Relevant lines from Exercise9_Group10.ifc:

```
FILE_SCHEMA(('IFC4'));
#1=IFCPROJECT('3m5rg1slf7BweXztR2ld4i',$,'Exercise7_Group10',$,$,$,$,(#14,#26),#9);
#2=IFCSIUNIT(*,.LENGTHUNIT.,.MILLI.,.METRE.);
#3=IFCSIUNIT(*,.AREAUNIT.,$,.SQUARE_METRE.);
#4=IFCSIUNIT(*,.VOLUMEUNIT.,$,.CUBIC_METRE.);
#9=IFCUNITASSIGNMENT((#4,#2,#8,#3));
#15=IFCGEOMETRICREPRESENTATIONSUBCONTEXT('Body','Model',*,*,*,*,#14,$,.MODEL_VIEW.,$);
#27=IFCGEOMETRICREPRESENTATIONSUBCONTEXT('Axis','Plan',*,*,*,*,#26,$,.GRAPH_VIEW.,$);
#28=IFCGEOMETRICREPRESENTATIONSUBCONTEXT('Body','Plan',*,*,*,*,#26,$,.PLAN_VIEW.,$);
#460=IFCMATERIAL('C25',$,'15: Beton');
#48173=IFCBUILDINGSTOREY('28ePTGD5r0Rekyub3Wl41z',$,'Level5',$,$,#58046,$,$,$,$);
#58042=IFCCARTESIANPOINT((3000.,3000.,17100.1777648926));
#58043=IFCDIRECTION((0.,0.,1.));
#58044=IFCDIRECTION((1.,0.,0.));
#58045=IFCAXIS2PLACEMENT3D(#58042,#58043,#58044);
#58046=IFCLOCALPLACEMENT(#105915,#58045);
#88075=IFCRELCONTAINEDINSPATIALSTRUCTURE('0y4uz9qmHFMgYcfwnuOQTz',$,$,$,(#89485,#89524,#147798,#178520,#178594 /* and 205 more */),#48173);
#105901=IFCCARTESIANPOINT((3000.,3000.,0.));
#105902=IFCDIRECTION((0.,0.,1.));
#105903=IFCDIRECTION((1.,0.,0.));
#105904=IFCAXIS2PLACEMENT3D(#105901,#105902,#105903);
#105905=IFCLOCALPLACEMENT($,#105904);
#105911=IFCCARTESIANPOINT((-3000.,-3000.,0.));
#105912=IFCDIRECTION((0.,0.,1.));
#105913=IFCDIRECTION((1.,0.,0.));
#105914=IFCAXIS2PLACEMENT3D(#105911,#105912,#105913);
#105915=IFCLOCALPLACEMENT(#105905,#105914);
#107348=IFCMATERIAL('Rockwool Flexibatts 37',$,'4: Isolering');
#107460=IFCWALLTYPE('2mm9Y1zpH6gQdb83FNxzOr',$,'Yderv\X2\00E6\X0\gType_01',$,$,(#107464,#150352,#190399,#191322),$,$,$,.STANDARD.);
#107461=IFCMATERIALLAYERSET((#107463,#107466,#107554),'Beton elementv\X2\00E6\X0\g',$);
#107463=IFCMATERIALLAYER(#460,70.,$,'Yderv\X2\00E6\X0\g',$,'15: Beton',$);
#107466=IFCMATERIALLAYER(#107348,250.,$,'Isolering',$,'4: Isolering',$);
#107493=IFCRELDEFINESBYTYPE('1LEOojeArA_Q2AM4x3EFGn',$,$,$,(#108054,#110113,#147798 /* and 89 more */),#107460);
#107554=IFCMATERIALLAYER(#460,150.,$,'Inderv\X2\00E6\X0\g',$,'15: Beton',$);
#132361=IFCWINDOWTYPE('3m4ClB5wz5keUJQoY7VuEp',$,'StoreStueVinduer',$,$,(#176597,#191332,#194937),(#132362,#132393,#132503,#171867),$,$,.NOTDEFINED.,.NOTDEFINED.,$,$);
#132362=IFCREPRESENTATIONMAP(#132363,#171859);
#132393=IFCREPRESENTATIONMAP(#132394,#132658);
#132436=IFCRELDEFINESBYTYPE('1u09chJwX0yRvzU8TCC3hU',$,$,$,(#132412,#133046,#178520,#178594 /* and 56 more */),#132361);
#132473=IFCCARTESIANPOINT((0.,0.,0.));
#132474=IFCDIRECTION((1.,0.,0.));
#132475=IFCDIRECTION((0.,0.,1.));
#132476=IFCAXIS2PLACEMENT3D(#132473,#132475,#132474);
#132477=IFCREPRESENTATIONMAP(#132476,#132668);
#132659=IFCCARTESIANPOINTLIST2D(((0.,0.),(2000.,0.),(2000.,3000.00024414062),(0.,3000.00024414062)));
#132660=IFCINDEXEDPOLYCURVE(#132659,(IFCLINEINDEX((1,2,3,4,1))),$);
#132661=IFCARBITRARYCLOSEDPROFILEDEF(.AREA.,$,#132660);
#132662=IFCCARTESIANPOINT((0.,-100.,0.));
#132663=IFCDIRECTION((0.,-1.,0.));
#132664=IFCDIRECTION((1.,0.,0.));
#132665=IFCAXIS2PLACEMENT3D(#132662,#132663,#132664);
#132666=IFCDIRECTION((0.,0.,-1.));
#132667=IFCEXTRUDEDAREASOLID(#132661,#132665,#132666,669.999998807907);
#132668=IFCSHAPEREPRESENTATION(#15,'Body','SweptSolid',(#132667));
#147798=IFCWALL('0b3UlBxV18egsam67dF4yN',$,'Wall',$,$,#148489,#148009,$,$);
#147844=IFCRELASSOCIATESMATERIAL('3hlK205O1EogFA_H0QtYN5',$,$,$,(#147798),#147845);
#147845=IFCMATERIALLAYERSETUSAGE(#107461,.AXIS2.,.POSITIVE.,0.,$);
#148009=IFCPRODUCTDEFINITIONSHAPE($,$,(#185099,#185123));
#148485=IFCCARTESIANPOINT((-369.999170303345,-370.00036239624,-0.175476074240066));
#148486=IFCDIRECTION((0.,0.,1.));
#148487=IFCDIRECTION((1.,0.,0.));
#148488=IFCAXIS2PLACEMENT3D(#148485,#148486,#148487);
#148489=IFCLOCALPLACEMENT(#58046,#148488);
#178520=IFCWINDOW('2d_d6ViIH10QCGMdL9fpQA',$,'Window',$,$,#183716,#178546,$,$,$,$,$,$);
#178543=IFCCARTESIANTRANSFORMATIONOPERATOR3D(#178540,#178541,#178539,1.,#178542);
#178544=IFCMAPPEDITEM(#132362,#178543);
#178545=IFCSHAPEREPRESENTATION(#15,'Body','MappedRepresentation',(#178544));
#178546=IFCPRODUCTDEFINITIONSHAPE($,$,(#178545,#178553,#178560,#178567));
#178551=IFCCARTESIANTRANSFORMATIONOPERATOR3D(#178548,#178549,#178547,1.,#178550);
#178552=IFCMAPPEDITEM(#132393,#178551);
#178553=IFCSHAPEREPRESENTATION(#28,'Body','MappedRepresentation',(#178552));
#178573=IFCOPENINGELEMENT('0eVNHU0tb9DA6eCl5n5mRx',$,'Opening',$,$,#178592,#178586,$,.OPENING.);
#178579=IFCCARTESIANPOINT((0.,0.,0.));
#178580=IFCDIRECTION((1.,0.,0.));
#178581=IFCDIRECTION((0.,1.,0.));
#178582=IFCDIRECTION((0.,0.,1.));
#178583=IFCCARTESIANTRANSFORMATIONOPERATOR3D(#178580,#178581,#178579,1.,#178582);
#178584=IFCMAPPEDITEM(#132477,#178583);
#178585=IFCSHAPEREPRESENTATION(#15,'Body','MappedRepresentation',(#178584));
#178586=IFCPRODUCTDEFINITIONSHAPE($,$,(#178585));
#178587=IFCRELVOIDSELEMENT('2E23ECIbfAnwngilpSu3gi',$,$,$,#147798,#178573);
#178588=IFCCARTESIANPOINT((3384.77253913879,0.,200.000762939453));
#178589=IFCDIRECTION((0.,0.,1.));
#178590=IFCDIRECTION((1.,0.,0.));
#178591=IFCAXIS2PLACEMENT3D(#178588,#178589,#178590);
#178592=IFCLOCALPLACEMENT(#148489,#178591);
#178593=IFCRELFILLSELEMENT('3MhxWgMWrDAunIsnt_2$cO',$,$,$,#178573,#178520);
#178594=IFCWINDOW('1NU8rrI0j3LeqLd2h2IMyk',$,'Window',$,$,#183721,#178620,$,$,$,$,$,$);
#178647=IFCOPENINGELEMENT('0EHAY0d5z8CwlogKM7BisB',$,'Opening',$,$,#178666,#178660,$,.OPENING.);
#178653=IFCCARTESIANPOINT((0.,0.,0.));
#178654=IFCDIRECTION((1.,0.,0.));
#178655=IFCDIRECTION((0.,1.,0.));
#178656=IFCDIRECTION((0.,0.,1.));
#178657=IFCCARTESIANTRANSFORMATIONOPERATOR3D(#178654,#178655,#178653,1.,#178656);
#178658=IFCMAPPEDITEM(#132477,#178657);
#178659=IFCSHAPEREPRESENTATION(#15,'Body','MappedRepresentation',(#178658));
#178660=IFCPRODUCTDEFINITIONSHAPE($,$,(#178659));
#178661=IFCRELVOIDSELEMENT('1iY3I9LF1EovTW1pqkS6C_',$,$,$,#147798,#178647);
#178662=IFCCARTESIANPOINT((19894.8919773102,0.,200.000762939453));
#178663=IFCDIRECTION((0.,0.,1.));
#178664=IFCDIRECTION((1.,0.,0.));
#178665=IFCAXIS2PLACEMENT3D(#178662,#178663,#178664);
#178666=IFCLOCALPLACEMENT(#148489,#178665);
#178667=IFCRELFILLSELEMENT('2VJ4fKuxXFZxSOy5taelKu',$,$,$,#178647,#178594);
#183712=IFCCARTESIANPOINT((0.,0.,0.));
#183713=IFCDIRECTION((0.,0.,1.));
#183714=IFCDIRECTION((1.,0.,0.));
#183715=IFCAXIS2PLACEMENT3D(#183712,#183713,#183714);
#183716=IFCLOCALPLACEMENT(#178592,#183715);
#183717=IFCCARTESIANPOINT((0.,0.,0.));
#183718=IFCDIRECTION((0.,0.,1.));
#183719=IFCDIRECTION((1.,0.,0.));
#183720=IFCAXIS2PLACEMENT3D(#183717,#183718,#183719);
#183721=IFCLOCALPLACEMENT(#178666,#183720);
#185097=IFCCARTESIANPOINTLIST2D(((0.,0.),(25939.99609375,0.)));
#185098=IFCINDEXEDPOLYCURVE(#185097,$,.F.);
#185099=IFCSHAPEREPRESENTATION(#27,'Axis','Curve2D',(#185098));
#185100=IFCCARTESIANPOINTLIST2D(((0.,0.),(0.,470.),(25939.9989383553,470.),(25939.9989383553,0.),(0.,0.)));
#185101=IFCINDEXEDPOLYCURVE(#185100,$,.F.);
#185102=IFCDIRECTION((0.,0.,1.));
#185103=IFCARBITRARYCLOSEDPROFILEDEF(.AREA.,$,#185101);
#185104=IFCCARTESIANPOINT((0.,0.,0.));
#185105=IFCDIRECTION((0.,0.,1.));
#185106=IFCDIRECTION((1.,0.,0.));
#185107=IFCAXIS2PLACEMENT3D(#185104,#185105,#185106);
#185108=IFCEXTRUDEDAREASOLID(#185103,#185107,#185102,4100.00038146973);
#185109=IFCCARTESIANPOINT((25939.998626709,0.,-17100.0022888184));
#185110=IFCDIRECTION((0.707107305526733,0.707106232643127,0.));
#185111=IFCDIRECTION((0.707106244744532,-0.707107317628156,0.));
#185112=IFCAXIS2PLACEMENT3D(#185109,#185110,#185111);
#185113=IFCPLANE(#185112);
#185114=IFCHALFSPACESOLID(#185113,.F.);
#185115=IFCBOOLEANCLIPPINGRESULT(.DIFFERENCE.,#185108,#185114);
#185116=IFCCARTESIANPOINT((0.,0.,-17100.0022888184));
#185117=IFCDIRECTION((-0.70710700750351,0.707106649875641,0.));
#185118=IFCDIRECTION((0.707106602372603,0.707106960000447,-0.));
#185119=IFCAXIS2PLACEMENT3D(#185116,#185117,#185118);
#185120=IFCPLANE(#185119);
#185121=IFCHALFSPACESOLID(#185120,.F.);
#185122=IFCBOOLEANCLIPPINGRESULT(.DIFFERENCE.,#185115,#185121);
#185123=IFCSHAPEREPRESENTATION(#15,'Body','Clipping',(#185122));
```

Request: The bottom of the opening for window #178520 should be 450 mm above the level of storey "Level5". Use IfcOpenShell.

```python
import numpy as np
import ifcopenshell
import ifcopenshell.api.geometry
import ifcopenshell.geom
import ifcopenshell.util.element
import ifcopenshell.util.placement
import ifcopenshell.util.shape
import ifcopenshell.util.unit

model = ifcopenshell.open("Exercise9_Group10.ifc")
unit_scale = ifcopenshell.util.unit.calculate_unit_scale(model)

window = model.by_id(178520)
opening = window.FillsVoids[0].RelatingOpeningElement
storey = ifcopenshell.util.element.get_container(window, ifc_class="IfcBuildingStorey")
level = ifcopenshell.util.placement.get_local_placement(storey.ObjectPlacement)[2, 3]

# The opening's origin need not be at the sill, so measure its lowest point.
shape = ifcopenshell.geom.create_shape(ifcopenshell.geom.settings(), opening)
bottom = ifcopenshell.util.shape.get_shape_bottom_elevation(shape, shape.geometry) / unit_scale
dz = level + 0.45 / unit_scale - bottom

shift = np.array([0.0, 0.0, dz])
# The window is placed relative to its opening, so it follows when the opening moves.
matrix = ifcopenshell.util.placement.get_local_placement(opening.ObjectPlacement)
matrix[:3, 3] += shift
ifcopenshell.api.geometry.edit_object_placement(
    model, product=opening, matrix=matrix, is_si=False, should_transform_children=True
)

print(f"moved by {dz * unit_scale:+.3f} m")

model.write("Exercise9_Group10_v2.ifc")
```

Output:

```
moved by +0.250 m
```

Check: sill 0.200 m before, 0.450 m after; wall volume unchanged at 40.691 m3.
